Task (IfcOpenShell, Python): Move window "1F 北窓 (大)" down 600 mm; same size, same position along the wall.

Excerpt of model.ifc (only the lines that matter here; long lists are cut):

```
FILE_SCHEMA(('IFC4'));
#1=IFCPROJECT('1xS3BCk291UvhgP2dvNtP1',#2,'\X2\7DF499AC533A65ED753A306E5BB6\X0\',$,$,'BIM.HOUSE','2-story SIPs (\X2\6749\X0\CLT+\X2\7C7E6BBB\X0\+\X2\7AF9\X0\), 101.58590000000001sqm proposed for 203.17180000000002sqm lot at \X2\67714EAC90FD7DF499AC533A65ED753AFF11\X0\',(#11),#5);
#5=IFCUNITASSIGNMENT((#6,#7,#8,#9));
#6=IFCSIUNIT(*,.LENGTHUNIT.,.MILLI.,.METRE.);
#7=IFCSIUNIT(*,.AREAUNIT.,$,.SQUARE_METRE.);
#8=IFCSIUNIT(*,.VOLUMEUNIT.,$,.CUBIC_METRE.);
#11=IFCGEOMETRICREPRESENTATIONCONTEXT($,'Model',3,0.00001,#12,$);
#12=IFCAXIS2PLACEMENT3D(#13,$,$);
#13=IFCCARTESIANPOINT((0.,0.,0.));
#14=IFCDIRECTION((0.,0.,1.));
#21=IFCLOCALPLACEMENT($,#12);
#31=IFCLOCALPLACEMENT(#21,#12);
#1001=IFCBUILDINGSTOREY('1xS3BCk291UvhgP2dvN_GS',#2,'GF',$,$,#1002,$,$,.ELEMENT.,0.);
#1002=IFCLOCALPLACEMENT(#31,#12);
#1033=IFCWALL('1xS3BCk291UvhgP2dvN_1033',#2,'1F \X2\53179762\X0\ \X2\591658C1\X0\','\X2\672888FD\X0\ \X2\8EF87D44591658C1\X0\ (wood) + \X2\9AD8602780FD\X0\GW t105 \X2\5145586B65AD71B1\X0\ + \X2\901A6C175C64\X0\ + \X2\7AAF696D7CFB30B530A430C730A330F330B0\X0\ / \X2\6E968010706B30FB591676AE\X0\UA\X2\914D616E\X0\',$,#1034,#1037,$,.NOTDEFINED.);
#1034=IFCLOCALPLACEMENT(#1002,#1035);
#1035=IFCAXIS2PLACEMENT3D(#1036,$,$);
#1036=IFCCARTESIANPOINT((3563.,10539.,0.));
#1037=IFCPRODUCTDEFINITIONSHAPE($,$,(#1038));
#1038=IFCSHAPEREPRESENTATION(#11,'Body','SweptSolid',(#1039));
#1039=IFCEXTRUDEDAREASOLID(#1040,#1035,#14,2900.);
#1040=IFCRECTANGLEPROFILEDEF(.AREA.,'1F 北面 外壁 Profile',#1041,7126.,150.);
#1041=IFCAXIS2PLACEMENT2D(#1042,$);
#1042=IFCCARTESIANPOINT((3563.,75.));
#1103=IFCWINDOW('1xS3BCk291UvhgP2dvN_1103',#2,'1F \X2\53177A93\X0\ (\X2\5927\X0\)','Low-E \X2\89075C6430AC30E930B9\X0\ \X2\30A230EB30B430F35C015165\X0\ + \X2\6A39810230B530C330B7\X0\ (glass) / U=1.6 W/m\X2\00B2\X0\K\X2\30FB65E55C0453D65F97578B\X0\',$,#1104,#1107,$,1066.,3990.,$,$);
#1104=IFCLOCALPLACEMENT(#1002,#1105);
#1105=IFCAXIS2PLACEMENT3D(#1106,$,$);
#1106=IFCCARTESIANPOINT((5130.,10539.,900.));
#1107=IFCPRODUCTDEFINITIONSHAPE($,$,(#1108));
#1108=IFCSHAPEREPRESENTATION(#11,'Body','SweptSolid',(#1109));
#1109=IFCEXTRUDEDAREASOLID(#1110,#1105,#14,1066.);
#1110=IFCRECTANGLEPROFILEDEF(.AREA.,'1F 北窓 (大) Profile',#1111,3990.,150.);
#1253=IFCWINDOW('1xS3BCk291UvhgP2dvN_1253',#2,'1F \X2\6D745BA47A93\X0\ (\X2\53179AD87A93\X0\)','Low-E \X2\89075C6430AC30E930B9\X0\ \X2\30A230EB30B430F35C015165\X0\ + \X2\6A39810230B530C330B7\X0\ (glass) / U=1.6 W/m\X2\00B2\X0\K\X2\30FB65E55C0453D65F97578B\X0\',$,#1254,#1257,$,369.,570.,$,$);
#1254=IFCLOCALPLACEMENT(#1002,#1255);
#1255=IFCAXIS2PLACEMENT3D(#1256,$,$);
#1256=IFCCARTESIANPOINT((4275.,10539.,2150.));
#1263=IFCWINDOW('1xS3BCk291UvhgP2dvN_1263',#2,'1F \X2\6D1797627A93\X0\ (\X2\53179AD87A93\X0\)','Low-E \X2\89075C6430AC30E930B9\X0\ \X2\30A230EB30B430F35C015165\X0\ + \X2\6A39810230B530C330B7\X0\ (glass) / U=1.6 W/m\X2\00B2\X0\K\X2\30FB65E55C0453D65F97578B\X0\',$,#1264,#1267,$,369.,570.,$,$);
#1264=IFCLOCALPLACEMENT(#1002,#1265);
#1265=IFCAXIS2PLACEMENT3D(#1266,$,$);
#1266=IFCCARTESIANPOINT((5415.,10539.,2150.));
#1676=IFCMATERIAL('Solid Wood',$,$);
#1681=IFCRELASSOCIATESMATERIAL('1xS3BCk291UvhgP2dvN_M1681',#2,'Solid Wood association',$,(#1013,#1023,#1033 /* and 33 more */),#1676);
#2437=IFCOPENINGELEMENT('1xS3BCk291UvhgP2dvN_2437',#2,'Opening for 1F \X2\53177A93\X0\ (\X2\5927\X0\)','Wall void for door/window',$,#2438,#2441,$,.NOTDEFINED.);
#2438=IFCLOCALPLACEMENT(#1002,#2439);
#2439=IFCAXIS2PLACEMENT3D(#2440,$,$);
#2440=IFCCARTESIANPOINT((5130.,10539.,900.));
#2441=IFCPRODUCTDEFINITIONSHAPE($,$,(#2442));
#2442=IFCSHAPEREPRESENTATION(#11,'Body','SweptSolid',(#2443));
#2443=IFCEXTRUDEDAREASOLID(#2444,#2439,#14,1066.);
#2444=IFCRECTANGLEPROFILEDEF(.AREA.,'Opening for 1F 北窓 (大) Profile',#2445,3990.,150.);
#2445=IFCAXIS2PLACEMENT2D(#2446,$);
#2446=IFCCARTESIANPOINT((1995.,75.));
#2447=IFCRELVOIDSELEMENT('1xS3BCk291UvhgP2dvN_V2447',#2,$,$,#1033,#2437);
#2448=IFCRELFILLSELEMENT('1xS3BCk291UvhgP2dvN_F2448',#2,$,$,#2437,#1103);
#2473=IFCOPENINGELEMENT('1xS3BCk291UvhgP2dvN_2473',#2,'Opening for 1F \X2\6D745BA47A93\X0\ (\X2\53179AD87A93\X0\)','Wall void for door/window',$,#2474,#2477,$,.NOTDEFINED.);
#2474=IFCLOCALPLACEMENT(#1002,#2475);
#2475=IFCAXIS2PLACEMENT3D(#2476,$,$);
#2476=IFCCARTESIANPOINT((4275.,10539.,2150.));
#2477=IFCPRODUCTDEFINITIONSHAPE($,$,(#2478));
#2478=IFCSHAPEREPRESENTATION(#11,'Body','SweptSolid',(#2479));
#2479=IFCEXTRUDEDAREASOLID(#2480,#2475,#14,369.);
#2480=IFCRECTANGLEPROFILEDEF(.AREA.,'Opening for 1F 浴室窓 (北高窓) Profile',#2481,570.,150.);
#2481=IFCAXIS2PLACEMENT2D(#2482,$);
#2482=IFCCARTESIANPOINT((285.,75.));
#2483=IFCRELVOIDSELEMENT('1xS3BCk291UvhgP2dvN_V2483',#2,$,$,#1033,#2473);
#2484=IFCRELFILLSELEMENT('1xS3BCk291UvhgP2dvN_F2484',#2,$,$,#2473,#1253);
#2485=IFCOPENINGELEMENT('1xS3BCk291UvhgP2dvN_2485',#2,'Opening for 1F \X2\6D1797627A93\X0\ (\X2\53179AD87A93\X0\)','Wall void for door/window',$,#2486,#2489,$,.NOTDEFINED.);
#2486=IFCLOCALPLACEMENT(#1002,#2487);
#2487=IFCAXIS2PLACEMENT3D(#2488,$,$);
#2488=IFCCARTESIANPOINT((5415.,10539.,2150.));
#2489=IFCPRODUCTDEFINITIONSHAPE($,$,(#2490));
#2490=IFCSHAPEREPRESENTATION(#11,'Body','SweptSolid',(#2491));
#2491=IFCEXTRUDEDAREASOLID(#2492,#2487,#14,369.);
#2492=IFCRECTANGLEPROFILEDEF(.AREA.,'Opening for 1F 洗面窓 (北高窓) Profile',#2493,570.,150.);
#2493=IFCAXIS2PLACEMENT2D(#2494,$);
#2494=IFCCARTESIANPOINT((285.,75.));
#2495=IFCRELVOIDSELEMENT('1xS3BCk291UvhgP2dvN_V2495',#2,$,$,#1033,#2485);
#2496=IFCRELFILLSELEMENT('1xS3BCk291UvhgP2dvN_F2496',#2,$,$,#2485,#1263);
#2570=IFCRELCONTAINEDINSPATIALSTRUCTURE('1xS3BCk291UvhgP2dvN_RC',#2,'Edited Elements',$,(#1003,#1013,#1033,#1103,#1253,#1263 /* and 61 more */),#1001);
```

```python
import numpy as np
import ifcopenshell
import ifcopenshell.api.geometry
import ifcopenshell.util.placement
import ifcopenshell.util.unit

model = ifcopenshell.open("model.ifc")
unit_scale = ifcopenshell.util.unit.calculate_unit_scale(model)

window = model.by_guid("1xS3BCk291UvhgP2dvN_1103")
opening = window.FillsVoids[0].RelatingOpeningElement
dz = -0.6 / unit_scale

shift = np.array([0.0, 0.0, dz])
# The window is not placed relative to its opening, so move both.
for product in (opening, window):
    matrix = ifcopenshell.util.placement.get_local_placement(product.ObjectPlacement)
    matrix[:3, 3] += shift
    ifcopenshell.api.geometry.edit_object_placement(model, product=product, matrix=matrix, is_si=False)

print(f"moved by {dz * unit_scale:+.3f} m")

model.write("model_rev.ifc")
```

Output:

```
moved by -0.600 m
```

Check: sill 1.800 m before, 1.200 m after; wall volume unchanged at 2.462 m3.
